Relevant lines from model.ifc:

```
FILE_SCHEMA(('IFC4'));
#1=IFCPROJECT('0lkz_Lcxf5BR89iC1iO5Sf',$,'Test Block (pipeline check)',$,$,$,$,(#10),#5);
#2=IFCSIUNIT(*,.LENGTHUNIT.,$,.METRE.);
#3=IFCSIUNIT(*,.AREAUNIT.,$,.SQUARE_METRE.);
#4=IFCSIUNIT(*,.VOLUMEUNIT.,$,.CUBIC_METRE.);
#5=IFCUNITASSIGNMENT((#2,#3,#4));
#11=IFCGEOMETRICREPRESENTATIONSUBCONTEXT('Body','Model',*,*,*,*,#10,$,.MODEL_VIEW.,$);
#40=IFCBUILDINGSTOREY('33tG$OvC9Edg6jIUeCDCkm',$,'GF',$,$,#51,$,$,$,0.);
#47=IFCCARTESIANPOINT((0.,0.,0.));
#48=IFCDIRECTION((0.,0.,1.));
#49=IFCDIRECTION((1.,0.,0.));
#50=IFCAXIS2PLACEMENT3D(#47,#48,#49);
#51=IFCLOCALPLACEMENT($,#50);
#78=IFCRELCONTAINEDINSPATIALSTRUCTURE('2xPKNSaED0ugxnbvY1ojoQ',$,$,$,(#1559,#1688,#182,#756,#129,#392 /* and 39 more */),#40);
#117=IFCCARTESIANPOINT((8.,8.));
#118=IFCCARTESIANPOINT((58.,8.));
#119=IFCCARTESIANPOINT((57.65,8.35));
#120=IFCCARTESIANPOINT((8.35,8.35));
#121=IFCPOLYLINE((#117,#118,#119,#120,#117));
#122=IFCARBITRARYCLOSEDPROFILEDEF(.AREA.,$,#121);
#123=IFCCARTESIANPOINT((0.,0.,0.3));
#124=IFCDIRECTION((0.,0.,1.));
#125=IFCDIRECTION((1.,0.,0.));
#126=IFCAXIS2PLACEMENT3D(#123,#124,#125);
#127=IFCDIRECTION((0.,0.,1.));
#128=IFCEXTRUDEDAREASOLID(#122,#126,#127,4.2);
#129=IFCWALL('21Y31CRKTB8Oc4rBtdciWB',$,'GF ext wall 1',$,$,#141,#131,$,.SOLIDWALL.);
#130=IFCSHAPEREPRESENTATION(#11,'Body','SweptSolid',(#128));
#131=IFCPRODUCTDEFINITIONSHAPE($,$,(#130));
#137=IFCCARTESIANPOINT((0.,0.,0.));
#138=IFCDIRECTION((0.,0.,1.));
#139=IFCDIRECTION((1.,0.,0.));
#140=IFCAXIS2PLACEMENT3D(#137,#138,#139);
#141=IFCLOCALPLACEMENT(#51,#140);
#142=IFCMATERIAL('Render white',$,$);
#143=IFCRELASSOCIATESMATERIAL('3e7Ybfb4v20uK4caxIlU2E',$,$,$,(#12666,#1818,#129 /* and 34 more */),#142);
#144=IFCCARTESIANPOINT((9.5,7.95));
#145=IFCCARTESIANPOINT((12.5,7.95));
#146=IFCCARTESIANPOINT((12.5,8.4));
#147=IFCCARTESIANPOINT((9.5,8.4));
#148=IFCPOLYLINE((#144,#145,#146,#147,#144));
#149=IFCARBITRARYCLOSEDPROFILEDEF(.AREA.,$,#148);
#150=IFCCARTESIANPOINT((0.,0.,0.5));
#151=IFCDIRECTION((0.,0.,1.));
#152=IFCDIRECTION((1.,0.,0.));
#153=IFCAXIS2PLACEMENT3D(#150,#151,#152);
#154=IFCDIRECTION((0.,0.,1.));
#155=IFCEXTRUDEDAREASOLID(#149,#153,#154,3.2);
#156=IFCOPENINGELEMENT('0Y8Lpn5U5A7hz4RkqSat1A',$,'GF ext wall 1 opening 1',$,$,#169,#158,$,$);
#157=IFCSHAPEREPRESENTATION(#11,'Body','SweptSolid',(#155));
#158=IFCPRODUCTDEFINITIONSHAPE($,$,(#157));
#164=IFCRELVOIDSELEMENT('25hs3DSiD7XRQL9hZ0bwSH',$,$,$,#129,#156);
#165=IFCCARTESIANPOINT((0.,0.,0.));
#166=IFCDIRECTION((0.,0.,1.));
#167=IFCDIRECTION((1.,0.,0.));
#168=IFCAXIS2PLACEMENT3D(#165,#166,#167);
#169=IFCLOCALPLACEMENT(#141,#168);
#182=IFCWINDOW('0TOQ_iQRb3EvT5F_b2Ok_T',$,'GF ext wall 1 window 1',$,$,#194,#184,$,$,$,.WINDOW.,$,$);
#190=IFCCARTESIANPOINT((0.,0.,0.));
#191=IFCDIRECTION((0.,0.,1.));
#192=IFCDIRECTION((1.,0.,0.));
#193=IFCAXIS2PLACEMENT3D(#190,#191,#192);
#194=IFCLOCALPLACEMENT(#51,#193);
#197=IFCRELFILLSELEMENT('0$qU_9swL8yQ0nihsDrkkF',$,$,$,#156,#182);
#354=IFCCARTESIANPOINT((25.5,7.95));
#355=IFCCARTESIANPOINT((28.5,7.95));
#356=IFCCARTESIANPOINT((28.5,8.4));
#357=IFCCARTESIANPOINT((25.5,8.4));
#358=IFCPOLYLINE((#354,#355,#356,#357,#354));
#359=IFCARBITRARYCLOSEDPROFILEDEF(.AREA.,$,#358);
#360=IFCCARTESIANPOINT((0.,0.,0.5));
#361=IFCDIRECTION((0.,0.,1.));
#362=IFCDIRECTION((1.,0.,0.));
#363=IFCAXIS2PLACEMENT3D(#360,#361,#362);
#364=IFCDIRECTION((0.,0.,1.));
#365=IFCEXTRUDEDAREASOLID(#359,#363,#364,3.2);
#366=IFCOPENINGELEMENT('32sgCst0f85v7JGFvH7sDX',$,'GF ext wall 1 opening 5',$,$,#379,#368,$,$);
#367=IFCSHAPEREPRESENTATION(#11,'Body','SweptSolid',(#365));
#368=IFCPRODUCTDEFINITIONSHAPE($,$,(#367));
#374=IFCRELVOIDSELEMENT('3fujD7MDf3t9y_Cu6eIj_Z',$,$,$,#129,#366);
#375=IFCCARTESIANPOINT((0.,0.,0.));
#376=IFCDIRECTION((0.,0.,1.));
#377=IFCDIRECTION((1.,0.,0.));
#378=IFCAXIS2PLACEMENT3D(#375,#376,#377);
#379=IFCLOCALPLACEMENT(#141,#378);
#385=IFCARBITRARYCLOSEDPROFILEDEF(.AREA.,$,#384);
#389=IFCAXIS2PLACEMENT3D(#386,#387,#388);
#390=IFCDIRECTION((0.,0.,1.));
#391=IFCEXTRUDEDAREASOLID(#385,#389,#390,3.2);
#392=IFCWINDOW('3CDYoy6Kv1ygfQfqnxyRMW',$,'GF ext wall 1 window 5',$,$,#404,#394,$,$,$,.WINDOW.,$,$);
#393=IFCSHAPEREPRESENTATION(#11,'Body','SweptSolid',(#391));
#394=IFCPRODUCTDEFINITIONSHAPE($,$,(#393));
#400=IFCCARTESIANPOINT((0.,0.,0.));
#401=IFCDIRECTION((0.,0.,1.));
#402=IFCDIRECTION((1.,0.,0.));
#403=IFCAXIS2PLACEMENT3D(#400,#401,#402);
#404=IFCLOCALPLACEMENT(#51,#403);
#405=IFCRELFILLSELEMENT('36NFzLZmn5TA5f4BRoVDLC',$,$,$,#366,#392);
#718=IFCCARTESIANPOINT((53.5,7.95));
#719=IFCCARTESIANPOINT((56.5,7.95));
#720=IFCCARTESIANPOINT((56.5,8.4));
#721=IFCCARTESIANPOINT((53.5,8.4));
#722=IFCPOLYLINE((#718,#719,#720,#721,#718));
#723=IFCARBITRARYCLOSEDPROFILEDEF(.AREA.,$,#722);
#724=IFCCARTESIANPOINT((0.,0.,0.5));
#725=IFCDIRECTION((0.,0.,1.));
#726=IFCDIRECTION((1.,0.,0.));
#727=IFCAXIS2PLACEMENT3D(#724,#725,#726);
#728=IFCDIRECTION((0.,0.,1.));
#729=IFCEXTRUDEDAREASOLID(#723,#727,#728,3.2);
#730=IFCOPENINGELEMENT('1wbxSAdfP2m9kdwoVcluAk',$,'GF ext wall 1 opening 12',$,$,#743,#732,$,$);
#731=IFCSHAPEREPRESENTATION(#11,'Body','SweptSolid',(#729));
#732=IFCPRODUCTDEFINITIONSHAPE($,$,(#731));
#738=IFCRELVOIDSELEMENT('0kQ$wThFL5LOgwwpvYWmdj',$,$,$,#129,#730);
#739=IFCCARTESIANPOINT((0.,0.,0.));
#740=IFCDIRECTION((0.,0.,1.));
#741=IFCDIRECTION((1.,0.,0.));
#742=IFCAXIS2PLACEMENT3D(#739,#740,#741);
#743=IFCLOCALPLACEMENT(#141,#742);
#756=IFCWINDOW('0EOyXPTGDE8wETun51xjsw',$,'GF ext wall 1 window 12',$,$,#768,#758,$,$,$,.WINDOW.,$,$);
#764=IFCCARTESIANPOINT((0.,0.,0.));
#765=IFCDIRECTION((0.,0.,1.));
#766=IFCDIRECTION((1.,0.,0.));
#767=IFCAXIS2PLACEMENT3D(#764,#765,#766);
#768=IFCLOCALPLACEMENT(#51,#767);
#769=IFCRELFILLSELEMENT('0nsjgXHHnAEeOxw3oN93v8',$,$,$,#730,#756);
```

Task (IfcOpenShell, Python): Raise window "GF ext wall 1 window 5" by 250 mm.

```python
import numpy as np
import ifcopenshell
import ifcopenshell.api.geometry
import ifcopenshell.util.placement
import ifcopenshell.util.unit

model = ifcopenshell.open("model.ifc")
unit_scale = ifcopenshell.util.unit.calculate_unit_scale(model)

window = model.by_id(392)
opening = window.FillsVoids[0].RelatingOpeningElement
dz = 0.25

shift = np.array([0.0, 0.0, dz])
# The window is not placed relative to its opening, so move both.
for product in (opening, window):
    matrix = ifcopenshell.util.placement.get_local_placement(product.ObjectPlacement)
    matrix[:3, 3] += shift
    ifcopenshell.api.geometry.edit_object_placement(model, product=product, matrix=matrix, is_si=False)

print(f"moved by {dz * unit_scale:+.3f} m")

model.write("model-out.ifc")
```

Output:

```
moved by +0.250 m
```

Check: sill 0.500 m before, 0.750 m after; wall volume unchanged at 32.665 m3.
